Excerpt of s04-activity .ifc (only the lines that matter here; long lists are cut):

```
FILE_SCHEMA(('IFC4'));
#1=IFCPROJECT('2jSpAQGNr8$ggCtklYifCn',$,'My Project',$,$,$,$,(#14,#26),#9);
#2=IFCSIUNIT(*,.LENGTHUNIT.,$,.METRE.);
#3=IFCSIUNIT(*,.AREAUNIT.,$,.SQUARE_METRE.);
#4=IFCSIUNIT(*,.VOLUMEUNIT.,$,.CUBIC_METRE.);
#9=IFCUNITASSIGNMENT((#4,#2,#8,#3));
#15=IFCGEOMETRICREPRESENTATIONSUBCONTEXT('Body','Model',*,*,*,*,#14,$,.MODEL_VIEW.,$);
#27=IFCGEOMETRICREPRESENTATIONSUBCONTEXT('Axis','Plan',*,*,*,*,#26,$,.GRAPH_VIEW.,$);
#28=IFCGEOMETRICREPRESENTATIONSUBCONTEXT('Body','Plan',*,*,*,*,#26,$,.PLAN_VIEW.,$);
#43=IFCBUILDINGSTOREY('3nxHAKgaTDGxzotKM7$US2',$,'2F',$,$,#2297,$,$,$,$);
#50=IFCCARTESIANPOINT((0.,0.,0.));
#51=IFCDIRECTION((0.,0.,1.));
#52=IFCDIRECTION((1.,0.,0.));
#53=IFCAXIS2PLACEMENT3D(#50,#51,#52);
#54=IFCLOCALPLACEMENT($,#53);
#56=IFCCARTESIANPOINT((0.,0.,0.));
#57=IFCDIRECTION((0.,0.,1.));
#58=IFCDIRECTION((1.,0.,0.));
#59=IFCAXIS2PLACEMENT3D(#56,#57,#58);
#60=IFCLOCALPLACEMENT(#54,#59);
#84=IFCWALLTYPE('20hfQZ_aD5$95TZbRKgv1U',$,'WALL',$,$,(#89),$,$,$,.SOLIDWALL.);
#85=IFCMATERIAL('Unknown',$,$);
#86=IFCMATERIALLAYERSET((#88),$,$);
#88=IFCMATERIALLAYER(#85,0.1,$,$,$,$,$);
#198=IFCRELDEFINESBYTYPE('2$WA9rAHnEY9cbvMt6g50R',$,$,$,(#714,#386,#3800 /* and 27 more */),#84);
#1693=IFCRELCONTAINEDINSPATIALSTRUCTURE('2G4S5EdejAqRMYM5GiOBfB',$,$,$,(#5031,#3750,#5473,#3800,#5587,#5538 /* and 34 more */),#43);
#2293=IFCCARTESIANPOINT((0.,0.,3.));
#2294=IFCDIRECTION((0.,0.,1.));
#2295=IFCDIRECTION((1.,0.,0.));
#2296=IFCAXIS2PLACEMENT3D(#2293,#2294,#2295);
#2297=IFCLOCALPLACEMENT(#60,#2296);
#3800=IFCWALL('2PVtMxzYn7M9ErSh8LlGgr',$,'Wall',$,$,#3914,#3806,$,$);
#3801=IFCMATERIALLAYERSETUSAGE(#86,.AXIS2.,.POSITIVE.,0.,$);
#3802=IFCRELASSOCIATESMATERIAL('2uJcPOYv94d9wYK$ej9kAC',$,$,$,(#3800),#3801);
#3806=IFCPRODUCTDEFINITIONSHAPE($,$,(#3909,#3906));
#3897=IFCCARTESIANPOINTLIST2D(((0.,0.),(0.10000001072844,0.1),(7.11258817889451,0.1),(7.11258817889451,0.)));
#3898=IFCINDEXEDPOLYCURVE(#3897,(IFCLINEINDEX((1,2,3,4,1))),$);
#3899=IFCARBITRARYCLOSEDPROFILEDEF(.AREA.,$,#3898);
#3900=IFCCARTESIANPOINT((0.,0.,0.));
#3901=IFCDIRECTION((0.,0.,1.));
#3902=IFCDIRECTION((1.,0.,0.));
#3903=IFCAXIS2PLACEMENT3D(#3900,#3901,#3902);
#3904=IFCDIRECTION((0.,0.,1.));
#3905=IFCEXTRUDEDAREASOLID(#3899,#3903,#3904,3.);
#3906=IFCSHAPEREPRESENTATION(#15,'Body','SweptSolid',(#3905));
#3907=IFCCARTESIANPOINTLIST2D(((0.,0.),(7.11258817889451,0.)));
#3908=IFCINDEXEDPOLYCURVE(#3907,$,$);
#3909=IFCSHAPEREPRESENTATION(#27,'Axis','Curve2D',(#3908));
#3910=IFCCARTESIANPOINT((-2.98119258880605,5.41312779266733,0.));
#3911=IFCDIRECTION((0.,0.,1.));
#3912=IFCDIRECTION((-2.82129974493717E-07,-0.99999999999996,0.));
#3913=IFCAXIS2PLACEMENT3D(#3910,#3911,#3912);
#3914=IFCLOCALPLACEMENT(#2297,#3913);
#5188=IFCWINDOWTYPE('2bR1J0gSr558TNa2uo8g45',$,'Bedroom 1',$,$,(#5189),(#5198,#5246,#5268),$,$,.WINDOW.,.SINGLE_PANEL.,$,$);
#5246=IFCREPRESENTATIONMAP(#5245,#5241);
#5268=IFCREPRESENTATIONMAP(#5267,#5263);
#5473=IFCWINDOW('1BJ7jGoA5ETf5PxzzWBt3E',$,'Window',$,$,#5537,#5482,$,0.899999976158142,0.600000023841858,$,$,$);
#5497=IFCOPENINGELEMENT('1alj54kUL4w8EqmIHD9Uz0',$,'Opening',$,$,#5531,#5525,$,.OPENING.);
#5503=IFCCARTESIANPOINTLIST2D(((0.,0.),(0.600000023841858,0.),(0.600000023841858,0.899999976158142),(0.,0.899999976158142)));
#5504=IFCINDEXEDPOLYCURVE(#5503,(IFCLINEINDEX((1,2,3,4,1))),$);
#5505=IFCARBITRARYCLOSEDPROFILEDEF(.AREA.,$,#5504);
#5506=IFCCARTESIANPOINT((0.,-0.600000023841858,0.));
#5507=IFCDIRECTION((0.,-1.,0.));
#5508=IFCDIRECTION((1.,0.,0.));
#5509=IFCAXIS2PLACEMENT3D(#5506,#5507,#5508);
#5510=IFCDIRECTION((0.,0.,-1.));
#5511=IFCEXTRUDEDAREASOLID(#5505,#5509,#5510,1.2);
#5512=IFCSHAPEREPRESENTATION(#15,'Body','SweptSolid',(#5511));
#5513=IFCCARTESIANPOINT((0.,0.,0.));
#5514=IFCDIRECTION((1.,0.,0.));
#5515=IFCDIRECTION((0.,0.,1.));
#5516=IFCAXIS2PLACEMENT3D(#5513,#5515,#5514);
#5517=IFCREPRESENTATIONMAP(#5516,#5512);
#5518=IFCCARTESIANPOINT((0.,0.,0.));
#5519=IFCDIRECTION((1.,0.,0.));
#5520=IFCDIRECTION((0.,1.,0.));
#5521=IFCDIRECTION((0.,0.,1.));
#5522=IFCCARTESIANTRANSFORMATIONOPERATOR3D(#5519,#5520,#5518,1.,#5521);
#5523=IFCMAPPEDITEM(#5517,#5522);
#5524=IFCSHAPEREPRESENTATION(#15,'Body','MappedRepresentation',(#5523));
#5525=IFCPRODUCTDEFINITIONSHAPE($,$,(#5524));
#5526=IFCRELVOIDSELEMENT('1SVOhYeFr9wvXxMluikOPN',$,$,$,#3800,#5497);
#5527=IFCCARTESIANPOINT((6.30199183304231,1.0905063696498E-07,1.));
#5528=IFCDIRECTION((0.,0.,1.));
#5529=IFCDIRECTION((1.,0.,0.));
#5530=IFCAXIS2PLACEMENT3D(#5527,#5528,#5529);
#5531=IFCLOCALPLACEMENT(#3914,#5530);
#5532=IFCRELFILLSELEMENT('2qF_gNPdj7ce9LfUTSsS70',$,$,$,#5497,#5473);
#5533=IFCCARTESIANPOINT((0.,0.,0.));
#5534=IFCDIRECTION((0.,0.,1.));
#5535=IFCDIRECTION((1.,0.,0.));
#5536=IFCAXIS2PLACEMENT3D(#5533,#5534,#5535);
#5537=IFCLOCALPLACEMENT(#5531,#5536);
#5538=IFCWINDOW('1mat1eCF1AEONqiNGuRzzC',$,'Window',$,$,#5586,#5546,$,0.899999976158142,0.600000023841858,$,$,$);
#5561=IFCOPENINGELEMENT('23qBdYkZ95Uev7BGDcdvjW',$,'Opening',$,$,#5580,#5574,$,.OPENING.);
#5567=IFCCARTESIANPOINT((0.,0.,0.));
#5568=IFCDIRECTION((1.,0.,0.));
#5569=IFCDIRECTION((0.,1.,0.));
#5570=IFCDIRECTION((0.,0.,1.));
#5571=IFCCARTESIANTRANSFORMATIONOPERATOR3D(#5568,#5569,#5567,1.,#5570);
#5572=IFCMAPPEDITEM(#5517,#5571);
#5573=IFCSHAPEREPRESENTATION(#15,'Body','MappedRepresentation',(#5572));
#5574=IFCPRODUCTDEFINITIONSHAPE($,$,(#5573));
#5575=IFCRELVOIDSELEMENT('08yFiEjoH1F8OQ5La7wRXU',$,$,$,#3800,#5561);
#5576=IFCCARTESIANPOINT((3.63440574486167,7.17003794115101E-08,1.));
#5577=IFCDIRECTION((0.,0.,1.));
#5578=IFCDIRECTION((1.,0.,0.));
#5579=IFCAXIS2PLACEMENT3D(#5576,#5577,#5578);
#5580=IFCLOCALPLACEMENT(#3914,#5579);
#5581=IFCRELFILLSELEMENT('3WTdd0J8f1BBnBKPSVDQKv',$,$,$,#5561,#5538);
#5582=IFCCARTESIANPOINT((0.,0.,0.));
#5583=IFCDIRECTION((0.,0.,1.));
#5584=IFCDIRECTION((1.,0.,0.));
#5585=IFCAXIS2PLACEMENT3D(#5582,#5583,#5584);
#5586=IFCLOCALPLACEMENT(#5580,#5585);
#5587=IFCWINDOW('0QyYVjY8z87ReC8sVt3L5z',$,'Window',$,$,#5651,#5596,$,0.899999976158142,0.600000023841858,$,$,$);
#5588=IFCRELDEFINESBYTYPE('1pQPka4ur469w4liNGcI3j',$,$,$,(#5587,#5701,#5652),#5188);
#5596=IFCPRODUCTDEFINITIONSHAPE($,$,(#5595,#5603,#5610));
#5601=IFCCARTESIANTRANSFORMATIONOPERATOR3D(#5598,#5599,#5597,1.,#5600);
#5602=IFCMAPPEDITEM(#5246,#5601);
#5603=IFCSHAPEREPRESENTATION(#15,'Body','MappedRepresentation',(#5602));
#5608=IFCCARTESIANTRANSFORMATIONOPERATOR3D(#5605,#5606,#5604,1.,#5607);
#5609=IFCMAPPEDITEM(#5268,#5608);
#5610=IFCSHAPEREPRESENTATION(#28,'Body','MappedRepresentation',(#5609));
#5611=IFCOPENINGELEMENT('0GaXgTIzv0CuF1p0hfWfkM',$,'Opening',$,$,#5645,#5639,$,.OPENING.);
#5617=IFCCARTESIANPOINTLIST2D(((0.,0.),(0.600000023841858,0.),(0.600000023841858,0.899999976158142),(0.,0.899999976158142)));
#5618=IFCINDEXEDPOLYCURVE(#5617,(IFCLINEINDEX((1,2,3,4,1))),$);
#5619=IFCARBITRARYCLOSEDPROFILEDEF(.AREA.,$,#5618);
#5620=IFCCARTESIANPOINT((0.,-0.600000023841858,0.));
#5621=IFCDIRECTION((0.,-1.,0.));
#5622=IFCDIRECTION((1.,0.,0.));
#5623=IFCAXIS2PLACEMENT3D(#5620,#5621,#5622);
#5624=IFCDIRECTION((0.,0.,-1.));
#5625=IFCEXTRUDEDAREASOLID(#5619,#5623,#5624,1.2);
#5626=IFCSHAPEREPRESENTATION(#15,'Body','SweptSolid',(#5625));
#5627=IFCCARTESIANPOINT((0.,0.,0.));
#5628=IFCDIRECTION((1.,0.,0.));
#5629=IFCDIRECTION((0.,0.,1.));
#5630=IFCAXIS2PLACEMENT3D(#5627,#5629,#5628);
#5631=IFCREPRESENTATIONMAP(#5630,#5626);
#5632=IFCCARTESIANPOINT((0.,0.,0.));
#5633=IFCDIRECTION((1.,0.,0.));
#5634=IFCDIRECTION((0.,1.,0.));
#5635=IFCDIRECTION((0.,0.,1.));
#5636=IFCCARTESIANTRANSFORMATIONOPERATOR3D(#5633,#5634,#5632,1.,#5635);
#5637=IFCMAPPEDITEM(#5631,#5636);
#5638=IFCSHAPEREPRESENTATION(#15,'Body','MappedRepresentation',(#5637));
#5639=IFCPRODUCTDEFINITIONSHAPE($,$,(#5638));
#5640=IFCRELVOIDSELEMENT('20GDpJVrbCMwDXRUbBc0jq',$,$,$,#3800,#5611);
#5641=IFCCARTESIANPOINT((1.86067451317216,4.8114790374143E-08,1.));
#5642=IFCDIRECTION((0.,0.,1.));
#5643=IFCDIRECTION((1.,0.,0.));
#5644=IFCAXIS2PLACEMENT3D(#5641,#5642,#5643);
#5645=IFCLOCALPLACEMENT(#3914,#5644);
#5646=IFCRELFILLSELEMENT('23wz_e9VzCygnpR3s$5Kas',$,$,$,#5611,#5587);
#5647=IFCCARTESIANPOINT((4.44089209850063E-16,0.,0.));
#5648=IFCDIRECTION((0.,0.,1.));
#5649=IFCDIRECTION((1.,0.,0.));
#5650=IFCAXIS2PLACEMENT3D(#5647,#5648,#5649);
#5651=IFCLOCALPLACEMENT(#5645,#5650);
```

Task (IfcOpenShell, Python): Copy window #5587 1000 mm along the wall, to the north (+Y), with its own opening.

```python
import ifcopenshell
import ifcopenshell.api.feature
import ifcopenshell.api.geometry
import ifcopenshell.api.root
import ifcopenshell.geom
import ifcopenshell.util.element
import ifcopenshell.util.placement
import ifcopenshell.util.shape
import ifcopenshell.util.unit

model = ifcopenshell.open("s04-activity .ifc")
unit_scale = ifcopenshell.util.unit.calculate_unit_scale(model)
settings = ifcopenshell.geom.settings()


def volume(element):
    """Net volume in cubic metres, openings subtracted."""
    shape = ifcopenshell.geom.create_shape(settings, element)
    return ifcopenshell.util.shape.get_volume(shape.geometry)


window = model.by_guid("0QyYVjY8z87ReC8sVt3L5z")
opening = window.FillsVoids[0].RelatingOpeningElement
wall = opening.VoidsElements[0].RelatingBuildingElement
before = volume(wall)
shift = ifcopenshell.util.placement.get_local_placement(wall.ObjectPlacement)[:3, 0] * -1 / unit_scale

# copy_class copies the void relationship, type, container and properties, but no geometry.
new_opening = ifcopenshell.api.root.copy_class(model, product=opening)
new_opening.Representation = ifcopenshell.util.element.copy_deep(
    model, opening.Representation, exclude=["IfcGeometricRepresentationContext", "IfcRepresentationMap"]
)
new_window = ifcopenshell.api.root.copy_class(model, product=window)
new_window.Representation = ifcopenshell.util.element.copy_deep(
    model, window.Representation, exclude=["IfcGeometricRepresentationContext", "IfcRepresentationMap"]
)
ifcopenshell.api.feature.add_filling(model, opening=new_opening, element=new_window)

for old, new in ((opening, new_opening), (window, new_window)):
    matrix = ifcopenshell.util.placement.get_local_placement(old.ObjectPlacement)
    matrix[:3, 3] += shift
    ifcopenshell.api.geometry.edit_object_placement(model, product=new, matrix=matrix, is_si=False)

after = volume(wall)

print(f"wall volume {before:.3f} -> {after:.3f} m3")

model.write("s04-activity -out.ifc")
```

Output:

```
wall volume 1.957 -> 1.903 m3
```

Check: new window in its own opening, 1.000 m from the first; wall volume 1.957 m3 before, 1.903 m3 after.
